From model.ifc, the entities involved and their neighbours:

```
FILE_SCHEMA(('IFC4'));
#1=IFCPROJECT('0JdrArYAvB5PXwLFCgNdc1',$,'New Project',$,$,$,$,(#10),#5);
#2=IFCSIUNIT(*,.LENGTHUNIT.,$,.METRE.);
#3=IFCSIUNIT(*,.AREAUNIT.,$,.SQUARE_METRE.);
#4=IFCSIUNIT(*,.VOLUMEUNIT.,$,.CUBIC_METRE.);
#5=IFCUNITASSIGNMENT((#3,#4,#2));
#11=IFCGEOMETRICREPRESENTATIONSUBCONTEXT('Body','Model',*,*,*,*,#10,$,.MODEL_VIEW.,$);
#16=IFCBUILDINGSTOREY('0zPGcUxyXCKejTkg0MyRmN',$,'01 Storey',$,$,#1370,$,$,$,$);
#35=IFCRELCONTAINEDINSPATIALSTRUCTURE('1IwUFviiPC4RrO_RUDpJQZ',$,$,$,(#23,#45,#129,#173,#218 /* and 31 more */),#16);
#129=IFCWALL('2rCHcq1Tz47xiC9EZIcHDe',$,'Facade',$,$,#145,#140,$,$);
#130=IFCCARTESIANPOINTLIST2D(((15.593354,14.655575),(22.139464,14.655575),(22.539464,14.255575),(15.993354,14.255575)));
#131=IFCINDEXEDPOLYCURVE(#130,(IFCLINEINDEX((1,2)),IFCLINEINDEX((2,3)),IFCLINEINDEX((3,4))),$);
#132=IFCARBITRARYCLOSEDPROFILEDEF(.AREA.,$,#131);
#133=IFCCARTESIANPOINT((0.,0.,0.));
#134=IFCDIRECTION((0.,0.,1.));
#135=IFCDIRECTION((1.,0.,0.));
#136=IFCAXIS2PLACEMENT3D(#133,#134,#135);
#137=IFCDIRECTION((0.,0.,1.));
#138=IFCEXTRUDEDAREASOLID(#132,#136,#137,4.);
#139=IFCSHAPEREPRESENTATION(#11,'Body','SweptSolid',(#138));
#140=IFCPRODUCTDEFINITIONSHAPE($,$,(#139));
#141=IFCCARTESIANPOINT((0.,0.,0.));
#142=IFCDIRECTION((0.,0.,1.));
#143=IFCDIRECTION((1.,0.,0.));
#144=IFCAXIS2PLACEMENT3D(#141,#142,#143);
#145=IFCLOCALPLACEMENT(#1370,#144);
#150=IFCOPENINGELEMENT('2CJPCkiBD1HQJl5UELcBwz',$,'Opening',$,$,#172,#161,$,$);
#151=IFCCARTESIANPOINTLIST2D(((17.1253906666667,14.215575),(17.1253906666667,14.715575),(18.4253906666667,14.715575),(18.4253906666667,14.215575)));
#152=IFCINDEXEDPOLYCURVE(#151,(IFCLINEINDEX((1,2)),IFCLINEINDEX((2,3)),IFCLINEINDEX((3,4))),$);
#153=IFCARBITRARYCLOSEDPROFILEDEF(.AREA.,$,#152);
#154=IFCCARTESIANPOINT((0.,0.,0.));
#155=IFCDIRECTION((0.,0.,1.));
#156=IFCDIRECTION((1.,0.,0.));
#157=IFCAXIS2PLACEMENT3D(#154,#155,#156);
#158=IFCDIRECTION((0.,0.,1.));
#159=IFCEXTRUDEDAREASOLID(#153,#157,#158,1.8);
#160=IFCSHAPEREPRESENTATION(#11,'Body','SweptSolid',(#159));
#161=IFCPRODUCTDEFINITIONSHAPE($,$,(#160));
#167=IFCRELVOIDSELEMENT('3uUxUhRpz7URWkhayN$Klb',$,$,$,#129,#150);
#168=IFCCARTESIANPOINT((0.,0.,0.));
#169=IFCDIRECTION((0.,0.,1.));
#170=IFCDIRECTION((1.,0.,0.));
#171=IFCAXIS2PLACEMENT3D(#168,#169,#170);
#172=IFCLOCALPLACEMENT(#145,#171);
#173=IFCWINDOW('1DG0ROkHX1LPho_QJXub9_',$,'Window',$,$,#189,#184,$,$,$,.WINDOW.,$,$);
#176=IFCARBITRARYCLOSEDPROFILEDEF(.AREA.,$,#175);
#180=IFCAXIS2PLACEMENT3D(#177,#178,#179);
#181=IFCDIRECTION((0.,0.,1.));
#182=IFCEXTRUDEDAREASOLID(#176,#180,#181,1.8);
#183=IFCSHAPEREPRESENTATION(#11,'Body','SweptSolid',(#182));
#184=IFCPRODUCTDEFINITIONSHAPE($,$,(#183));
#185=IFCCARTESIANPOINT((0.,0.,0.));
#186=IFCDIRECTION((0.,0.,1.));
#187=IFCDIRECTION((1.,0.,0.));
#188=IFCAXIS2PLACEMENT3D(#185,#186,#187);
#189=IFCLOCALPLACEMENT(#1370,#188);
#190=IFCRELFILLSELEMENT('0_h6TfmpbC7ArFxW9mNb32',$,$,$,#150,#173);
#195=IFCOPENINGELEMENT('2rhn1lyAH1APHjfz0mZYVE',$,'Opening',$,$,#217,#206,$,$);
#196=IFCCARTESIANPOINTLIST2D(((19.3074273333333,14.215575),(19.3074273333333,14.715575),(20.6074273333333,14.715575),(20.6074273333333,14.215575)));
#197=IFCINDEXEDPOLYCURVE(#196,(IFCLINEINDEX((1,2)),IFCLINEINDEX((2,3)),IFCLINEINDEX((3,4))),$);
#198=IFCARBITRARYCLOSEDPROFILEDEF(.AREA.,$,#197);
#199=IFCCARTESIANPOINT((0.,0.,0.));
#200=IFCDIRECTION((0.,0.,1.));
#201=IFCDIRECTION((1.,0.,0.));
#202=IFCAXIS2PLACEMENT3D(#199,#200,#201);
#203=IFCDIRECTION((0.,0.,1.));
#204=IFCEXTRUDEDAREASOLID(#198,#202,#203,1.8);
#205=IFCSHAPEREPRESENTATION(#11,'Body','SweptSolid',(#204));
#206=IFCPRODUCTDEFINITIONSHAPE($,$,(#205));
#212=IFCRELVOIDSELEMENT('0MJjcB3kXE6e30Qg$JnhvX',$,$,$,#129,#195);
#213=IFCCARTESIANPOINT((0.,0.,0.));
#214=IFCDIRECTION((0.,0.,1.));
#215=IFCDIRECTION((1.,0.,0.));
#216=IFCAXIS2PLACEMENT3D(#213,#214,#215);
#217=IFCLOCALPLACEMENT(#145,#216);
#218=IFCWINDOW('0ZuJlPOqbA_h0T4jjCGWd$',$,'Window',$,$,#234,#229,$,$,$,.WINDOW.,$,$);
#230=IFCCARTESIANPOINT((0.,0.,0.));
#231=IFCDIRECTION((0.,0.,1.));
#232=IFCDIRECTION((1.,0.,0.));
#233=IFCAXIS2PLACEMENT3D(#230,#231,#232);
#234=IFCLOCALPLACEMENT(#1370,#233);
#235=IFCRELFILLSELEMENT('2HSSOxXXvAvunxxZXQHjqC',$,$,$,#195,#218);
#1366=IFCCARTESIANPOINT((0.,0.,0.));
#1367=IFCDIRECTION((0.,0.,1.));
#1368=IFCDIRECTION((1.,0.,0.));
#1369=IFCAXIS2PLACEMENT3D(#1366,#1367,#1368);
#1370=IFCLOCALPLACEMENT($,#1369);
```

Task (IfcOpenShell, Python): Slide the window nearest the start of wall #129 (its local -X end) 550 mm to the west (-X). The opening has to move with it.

```python
import ifcopenshell
import ifcopenshell.api.geometry
import ifcopenshell.util.placement
import ifcopenshell.util.unit

model = ifcopenshell.open("model.ifc")
unit_scale = ifcopenshell.util.unit.calculate_unit_scale(model)

window = model.by_guid("1DG0ROkHX1LPho_QJXub9_")
opening = window.FillsVoids[0].RelatingOpeningElement
wall = opening.VoidsElements[0].RelatingBuildingElement

wall_matrix = ifcopenshell.util.placement.get_local_placement(wall.ObjectPlacement)
shift = wall_matrix[:3, 0] * -0.55 / unit_scale
before = ifcopenshell.util.placement.get_local_placement(window.ObjectPlacement)[:3, 3].copy()

# The window is not placed relative to its opening, so move both.
for product in (opening, window):
    matrix = ifcopenshell.util.placement.get_local_placement(product.ObjectPlacement)
    matrix[:3, 3] += shift
    ifcopenshell.api.geometry.edit_object_placement(model, product=product, matrix=matrix, is_si=False)

after = ifcopenshell.util.placement.get_local_placement(window.ObjectPlacement)[:3, 3]
print("window moved by", (after - before).round(3) + 0.0)

model.write("model_v2.ifc")
```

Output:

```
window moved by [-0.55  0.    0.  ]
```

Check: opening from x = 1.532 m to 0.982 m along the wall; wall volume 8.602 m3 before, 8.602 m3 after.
